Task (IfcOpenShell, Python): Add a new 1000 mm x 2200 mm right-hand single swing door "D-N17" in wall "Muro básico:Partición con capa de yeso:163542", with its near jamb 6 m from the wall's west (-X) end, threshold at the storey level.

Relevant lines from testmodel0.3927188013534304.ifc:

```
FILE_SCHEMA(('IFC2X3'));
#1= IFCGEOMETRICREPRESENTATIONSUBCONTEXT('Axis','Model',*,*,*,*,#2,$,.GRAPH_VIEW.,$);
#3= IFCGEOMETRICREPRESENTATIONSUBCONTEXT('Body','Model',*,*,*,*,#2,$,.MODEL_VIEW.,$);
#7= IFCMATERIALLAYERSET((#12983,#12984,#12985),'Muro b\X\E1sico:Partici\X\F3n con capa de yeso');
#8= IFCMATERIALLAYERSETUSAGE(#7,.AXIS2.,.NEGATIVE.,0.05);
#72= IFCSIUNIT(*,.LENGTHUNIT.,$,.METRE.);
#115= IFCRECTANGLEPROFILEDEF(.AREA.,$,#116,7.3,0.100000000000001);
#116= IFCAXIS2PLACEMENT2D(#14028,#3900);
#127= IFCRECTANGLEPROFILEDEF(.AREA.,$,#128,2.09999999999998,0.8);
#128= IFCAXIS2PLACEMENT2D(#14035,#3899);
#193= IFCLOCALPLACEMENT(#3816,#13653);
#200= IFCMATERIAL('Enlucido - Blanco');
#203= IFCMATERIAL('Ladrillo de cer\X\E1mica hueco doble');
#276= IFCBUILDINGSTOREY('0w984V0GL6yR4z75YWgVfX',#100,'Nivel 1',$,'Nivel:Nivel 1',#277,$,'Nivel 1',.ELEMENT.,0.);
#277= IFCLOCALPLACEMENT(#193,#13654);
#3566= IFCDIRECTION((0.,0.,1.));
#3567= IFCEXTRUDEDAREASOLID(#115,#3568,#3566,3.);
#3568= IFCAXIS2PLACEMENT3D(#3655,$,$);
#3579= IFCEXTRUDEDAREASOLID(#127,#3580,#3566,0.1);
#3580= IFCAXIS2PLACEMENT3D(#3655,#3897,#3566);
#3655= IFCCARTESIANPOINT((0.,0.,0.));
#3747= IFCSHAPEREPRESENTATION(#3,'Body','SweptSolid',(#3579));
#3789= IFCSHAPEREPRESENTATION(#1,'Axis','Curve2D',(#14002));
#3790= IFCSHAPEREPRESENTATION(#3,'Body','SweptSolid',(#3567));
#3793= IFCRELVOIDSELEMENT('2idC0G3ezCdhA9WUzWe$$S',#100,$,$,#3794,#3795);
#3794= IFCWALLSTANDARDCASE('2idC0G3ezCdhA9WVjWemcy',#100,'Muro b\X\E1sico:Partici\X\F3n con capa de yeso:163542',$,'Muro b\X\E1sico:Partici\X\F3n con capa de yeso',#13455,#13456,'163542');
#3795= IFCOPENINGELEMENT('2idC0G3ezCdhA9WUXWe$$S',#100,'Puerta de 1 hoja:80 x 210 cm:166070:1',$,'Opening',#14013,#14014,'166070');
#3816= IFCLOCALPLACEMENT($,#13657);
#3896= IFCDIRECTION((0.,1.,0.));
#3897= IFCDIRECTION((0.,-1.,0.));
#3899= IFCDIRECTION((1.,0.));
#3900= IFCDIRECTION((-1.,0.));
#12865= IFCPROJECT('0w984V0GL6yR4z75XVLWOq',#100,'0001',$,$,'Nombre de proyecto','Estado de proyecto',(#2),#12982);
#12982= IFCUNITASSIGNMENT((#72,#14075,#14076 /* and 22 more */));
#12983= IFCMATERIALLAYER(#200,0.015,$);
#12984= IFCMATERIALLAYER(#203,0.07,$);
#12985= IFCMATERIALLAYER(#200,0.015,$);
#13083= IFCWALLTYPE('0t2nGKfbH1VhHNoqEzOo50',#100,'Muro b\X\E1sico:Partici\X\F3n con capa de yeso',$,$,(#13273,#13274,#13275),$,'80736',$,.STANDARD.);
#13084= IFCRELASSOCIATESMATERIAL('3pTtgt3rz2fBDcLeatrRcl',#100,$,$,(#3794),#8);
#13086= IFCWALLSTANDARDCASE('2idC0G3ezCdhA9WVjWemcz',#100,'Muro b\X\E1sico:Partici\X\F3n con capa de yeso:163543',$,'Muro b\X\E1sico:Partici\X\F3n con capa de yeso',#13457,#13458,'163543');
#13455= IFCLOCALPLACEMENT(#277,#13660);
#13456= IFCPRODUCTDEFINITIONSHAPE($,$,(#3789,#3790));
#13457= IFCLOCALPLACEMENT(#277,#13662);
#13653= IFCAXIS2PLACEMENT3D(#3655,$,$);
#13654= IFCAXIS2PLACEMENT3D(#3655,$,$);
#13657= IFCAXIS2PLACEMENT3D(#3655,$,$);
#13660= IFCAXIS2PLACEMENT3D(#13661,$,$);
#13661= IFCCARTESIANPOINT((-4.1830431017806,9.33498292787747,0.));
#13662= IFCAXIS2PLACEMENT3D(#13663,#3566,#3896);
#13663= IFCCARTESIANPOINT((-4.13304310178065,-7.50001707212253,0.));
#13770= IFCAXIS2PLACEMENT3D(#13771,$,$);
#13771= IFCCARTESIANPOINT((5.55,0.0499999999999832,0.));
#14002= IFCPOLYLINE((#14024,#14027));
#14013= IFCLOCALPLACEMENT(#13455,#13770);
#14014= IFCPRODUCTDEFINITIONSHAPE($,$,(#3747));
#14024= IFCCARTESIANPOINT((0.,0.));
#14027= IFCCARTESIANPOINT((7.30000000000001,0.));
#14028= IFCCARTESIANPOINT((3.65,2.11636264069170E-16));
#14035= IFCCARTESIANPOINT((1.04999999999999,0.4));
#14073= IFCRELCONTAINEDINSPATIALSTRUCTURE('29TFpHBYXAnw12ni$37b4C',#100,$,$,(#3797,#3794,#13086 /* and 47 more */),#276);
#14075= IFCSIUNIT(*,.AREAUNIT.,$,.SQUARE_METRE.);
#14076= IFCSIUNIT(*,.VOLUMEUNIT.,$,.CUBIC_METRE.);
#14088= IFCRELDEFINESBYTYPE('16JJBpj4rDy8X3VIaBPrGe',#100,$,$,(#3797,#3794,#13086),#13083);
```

```python
import numpy as np
import ifcopenshell
import ifcopenshell.api.feature
import ifcopenshell.api.geometry
import ifcopenshell.api.root
import ifcopenshell.api.spatial
import ifcopenshell.api.type
import ifcopenshell.geom
import ifcopenshell.util.element
import ifcopenshell.util.placement
import ifcopenshell.util.representation
import ifcopenshell.util.shape
import ifcopenshell.util.unit

model = ifcopenshell.open("testmodel0.3927188013534304.ifc")
unit_scale = ifcopenshell.util.unit.calculate_unit_scale(model)
settings = ifcopenshell.geom.settings()


def volume(element):
    """Net volume in cubic metres, openings subtracted."""
    shape = ifcopenshell.geom.create_shape(settings, element)
    return ifcopenshell.util.shape.get_volume(shape.geometry)


wall = model.by_guid("2idC0G3ezCdhA9WVjWemcy")
storey = ifcopenshell.util.element.get_container(wall, ifc_class="IfcBuildingStorey")
context = ifcopenshell.util.representation.get_context(model, "Model", "Body", "MODEL_VIEW")
before = volume(wall)

width, height, from_end, sill = 1, 2.2, 6, 0.0  # metres

# The wall runs along its own X axis, and the end named is its -X end.
wall_shape = ifcopenshell.geom.create_shape(settings, wall)
x, y, z = ifcopenshell.util.shape.get_vertices(wall_shape.geometry).T
start = x.min() + from_end
face, thickness = float(y.min()), float(y.max() - y.min())
wall_matrix = ifcopenshell.util.placement.get_local_placement(wall.ObjectPlacement)
level = ifcopenshell.util.placement.get_local_placement(storey.ObjectPlacement)[2, 3]


def in_wall(x, y):
    """Placement at x, y metres in the wall's axes, at sill height."""
    matrix = wall_matrix.copy()
    matrix[:, 3] = wall_matrix @ np.array([x / unit_scale, y / unit_scale, 0.0, 1.0])
    matrix[2, 3] = level + sill / unit_scale
    return matrix


# Opening: a box that overshoots both wall faces by 50 mm.
opening = ifcopenshell.api.root.create_entity(model, ifc_class="IfcOpeningElement")
box = ifcopenshell.api.geometry.add_wall_representation(
    model, context=context, length=width, height=height, thickness=thickness + 0.1
)
ifcopenshell.api.geometry.assign_representation(model, product=opening, representation=box)
ifcopenshell.api.geometry.edit_object_placement(model, product=opening, matrix=in_wall(start, face - 0.05), is_si=False)
ifcopenshell.api.feature.add_feature(model, feature=opening, element=wall)

door = ifcopenshell.api.root.create_entity(model, ifc_class="IfcDoor", name="D-N17")
door.OverallWidth, door.OverallHeight = width / unit_scale, height / unit_scale
body = ifcopenshell.api.geometry.add_door_representation(
    model,
    context=context,
    overall_width=door.OverallWidth,
    overall_height=door.OverallHeight,
    operation_type="SINGLE_SWING_RIGHT",
    lining_properties={"LiningDepth": thickness / unit_scale, "ThresholdDepth": thickness / unit_scale},
)
ifcopenshell.api.geometry.assign_representation(model, product=door, representation=body)
ifcopenshell.api.spatial.assign_container(model, products=[door], relating_structure=storey)
fills = ifcopenshell.api.feature.add_filling(model, opening=opening, element=door)
fills.OwnerHistory = door.OwnerHistory  # required in IFC2X3

# IFC2X3 keeps the operation on the door style.
style = ifcopenshell.api.root.create_entity(model, ifc_class="IfcDoorStyle", name="D-N17")
style.OperationType, style.ConstructionType = "SINGLE_SWING_RIGHT", "NOTDEFINED"
style.ParameterTakesPrecedence = style.Sizeable = False
ifcopenshell.api.type.assign_type(model, related_objects=[door], relating_type=style)

# The lining spans the wall, so the door starts at the wall face.
ifcopenshell.api.geometry.edit_object_placement(model, product=door, matrix=in_wall(start, face), is_si=False)

after = volume(wall)

print(f"wall volume {before:.3f} -> {after:.3f} m3")

model.write("testmodel0.3927188013534304_rev.ifc")
```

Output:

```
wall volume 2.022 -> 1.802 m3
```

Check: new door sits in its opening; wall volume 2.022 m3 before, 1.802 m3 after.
